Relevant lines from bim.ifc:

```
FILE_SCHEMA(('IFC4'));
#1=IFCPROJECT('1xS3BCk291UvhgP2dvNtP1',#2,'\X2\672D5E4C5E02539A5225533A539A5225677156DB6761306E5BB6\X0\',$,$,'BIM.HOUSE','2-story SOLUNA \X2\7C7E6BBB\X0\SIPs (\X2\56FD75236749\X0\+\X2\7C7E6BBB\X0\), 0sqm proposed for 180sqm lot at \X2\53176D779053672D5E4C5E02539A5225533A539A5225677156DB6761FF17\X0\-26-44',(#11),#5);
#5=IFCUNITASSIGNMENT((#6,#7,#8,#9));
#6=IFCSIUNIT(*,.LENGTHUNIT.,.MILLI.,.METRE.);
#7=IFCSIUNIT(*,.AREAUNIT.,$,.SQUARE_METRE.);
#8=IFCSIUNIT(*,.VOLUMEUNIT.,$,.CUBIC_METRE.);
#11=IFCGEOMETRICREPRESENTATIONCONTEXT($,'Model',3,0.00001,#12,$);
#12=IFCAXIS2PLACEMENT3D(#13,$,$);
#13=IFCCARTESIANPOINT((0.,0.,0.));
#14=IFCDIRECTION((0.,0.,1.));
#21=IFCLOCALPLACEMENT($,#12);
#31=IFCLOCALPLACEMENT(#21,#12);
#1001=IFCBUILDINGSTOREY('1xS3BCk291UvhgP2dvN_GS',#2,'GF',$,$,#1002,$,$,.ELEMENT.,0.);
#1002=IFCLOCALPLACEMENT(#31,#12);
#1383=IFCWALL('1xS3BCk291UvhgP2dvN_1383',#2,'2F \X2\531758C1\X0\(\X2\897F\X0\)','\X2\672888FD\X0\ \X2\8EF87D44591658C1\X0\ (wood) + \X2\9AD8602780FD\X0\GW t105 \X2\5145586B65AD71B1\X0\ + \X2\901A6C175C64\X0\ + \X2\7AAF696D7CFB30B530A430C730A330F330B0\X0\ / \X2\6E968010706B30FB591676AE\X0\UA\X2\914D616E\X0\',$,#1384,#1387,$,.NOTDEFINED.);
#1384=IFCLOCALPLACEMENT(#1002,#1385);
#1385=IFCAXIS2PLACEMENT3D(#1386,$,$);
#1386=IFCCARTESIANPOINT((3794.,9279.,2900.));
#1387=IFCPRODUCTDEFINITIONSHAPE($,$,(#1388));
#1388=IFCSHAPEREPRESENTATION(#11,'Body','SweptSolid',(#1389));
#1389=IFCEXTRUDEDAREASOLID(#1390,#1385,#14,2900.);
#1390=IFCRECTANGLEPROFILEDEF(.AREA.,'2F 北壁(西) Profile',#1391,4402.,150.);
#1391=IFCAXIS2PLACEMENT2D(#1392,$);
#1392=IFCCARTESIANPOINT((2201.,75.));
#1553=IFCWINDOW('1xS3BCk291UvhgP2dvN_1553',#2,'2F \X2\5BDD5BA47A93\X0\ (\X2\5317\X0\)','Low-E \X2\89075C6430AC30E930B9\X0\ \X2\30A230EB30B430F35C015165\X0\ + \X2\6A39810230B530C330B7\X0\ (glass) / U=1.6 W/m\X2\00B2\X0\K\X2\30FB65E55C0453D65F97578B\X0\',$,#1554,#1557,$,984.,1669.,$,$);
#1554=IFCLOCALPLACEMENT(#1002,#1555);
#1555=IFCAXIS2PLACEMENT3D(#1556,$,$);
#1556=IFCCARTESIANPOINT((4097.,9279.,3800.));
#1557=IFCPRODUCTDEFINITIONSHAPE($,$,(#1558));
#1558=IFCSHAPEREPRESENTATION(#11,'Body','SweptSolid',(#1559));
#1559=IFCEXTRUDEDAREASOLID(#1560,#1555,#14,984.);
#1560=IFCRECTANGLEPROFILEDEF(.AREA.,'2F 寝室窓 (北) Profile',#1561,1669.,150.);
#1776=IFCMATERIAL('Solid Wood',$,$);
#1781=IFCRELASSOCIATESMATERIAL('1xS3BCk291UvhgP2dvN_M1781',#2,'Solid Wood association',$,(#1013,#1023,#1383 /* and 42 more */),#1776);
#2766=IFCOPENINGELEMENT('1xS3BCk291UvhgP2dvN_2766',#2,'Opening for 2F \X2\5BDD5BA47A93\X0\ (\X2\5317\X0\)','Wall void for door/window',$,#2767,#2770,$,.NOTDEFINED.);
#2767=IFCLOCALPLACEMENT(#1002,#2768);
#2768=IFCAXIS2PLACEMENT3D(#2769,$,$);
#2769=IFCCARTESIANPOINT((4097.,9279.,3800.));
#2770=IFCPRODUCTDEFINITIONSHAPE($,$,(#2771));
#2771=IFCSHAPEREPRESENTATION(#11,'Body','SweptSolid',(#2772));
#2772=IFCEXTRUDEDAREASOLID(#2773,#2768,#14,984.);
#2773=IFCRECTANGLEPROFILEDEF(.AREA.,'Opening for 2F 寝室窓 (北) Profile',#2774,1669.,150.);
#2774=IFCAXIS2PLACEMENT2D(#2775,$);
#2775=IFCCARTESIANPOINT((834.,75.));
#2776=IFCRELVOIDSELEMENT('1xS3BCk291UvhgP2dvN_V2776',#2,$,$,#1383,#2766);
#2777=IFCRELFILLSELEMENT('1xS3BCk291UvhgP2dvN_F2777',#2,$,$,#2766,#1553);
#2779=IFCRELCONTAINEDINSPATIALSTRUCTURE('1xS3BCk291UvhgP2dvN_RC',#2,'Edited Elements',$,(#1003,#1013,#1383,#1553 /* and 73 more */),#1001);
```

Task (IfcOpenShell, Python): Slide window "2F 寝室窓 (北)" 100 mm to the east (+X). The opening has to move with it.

```python
import ifcopenshell
import ifcopenshell.api.geometry
import ifcopenshell.util.placement
import ifcopenshell.util.unit

model = ifcopenshell.open("bim.ifc")
unit_scale = ifcopenshell.util.unit.calculate_unit_scale(model)

window = model.by_id(1553)
opening = window.FillsVoids[0].RelatingOpeningElement
wall = opening.VoidsElements[0].RelatingBuildingElement

wall_matrix = ifcopenshell.util.placement.get_local_placement(wall.ObjectPlacement)
shift = wall_matrix[:3, 0] * 0.1 / unit_scale
before = ifcopenshell.util.placement.get_local_placement(window.ObjectPlacement)[:3, 3].copy()

# The window is not placed relative to its opening, so move both.
for product in (opening, window):
    matrix = ifcopenshell.util.placement.get_local_placement(product.ObjectPlacement)
    matrix[:3, 3] += shift
    ifcopenshell.api.geometry.edit_object_placement(model, product=product, matrix=matrix, is_si=False)

after = ifcopenshell.util.placement.get_local_placement(window.ObjectPlacement)[:3, 3]
print("window moved by", (after - before).round(3) + 0.0)

model.write("bim_rev.ifc")
```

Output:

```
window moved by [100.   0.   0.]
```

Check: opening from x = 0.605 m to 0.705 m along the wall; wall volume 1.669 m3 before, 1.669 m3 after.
